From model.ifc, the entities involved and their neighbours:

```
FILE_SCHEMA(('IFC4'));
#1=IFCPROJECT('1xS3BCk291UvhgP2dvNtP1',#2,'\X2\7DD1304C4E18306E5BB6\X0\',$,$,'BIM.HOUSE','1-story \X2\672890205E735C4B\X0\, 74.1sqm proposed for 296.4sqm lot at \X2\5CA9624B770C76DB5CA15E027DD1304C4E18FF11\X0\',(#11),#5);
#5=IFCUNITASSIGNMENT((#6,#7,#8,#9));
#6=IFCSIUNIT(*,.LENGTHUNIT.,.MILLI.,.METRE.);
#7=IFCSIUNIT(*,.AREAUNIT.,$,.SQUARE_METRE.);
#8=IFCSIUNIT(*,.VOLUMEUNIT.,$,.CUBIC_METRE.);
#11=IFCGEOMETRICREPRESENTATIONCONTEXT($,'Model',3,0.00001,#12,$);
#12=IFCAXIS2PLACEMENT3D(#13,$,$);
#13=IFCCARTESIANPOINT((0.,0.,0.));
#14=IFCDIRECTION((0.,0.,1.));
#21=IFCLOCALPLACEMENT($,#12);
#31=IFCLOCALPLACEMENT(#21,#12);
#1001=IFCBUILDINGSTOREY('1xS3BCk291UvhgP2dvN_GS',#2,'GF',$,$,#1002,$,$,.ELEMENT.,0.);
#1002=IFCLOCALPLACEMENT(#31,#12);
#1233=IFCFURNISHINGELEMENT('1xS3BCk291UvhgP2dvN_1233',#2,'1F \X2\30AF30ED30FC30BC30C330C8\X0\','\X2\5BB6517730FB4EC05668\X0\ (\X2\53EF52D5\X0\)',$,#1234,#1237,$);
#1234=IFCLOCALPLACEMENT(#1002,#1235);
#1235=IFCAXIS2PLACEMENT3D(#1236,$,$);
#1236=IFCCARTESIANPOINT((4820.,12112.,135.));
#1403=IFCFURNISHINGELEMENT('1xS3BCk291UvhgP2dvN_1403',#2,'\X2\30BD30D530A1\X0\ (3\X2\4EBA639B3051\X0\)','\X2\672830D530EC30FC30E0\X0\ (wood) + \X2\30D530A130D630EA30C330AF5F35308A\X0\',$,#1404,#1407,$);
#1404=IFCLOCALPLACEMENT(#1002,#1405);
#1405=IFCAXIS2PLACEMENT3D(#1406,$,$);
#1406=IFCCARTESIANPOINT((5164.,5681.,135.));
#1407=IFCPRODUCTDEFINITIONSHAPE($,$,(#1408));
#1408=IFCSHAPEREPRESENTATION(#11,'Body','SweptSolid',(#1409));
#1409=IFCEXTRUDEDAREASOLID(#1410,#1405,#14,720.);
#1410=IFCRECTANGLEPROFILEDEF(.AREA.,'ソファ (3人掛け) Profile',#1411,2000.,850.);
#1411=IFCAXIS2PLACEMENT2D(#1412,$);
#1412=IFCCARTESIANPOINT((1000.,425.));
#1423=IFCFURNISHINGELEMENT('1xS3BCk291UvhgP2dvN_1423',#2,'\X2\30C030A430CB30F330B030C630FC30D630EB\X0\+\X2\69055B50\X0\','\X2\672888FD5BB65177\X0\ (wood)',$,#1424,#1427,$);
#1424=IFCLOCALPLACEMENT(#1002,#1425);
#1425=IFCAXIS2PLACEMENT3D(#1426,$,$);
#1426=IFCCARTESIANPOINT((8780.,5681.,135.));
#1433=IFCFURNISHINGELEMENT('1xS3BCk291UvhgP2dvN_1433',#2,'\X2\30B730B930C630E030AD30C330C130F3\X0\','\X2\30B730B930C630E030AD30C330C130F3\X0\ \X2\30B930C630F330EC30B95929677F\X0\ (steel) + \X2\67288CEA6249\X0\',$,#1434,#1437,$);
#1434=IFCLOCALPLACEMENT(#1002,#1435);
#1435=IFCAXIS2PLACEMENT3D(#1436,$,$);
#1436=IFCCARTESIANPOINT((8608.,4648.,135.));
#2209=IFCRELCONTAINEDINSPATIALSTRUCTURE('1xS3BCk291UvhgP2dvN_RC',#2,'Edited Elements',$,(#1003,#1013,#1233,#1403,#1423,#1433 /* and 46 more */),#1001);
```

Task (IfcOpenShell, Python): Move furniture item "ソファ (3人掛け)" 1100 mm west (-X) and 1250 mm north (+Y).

```python
import ifcopenshell
import ifcopenshell.api.geometry
import ifcopenshell.util.placement
import ifcopenshell.util.unit

model = ifcopenshell.open("model.ifc")
unit_scale = ifcopenshell.util.unit.calculate_unit_scale(model)

item = model.by_guid("1xS3BCk291UvhgP2dvN_1403")
matrix = ifcopenshell.util.placement.get_local_placement(item.ObjectPlacement)
matrix[0, 3] -= 1.1 / unit_scale
matrix[1, 3] += 1.25 / unit_scale
ifcopenshell.api.geometry.edit_object_placement(model, product=item, matrix=matrix, is_si=False)

print(ifcopenshell.util.placement.get_local_placement(item.ObjectPlacement).round(3) + 0.0)

model.write("model-out.ifc")
```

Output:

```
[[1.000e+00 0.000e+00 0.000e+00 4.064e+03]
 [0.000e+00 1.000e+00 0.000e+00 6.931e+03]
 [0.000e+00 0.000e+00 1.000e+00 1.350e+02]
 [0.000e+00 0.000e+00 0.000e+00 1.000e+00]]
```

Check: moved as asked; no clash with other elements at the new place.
